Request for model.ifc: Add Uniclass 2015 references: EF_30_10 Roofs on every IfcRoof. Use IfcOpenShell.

First a look at what the model holds.

```python
import ifcopenshell

model = ifcopenshell.open("model.ifc")
print(model.schema)
print("classifications:", [c.Name for c in model.by_type("IfcClassification")])
for ifc_class in ("IfcDoor", "IfcRoof", "IfcStair", "IfcWall", "IfcWindow"):
    print(ifc_class, len(model.by_type(ifc_class)))
```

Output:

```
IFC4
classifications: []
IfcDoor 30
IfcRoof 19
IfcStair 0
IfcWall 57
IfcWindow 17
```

```python
import ifcopenshell
import ifcopenshell.api.classification

model = ifcopenshell.open("model.ifc")

system = ifcopenshell.api.classification.add_classification(model, classification="Uniclass 2015")

codes = {
    "IfcRoof": ("EF_30_10", "Roofs"),
}
for ifc_class, (code, name) in codes.items():
    products = model.by_type(ifc_class)
    ifcopenshell.api.classification.add_reference(
        model, products=products, classification=system, identification=code, name=name
    )
    print(code, len(products))

model.write("model_rev.ifc")
```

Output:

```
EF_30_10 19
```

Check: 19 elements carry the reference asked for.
